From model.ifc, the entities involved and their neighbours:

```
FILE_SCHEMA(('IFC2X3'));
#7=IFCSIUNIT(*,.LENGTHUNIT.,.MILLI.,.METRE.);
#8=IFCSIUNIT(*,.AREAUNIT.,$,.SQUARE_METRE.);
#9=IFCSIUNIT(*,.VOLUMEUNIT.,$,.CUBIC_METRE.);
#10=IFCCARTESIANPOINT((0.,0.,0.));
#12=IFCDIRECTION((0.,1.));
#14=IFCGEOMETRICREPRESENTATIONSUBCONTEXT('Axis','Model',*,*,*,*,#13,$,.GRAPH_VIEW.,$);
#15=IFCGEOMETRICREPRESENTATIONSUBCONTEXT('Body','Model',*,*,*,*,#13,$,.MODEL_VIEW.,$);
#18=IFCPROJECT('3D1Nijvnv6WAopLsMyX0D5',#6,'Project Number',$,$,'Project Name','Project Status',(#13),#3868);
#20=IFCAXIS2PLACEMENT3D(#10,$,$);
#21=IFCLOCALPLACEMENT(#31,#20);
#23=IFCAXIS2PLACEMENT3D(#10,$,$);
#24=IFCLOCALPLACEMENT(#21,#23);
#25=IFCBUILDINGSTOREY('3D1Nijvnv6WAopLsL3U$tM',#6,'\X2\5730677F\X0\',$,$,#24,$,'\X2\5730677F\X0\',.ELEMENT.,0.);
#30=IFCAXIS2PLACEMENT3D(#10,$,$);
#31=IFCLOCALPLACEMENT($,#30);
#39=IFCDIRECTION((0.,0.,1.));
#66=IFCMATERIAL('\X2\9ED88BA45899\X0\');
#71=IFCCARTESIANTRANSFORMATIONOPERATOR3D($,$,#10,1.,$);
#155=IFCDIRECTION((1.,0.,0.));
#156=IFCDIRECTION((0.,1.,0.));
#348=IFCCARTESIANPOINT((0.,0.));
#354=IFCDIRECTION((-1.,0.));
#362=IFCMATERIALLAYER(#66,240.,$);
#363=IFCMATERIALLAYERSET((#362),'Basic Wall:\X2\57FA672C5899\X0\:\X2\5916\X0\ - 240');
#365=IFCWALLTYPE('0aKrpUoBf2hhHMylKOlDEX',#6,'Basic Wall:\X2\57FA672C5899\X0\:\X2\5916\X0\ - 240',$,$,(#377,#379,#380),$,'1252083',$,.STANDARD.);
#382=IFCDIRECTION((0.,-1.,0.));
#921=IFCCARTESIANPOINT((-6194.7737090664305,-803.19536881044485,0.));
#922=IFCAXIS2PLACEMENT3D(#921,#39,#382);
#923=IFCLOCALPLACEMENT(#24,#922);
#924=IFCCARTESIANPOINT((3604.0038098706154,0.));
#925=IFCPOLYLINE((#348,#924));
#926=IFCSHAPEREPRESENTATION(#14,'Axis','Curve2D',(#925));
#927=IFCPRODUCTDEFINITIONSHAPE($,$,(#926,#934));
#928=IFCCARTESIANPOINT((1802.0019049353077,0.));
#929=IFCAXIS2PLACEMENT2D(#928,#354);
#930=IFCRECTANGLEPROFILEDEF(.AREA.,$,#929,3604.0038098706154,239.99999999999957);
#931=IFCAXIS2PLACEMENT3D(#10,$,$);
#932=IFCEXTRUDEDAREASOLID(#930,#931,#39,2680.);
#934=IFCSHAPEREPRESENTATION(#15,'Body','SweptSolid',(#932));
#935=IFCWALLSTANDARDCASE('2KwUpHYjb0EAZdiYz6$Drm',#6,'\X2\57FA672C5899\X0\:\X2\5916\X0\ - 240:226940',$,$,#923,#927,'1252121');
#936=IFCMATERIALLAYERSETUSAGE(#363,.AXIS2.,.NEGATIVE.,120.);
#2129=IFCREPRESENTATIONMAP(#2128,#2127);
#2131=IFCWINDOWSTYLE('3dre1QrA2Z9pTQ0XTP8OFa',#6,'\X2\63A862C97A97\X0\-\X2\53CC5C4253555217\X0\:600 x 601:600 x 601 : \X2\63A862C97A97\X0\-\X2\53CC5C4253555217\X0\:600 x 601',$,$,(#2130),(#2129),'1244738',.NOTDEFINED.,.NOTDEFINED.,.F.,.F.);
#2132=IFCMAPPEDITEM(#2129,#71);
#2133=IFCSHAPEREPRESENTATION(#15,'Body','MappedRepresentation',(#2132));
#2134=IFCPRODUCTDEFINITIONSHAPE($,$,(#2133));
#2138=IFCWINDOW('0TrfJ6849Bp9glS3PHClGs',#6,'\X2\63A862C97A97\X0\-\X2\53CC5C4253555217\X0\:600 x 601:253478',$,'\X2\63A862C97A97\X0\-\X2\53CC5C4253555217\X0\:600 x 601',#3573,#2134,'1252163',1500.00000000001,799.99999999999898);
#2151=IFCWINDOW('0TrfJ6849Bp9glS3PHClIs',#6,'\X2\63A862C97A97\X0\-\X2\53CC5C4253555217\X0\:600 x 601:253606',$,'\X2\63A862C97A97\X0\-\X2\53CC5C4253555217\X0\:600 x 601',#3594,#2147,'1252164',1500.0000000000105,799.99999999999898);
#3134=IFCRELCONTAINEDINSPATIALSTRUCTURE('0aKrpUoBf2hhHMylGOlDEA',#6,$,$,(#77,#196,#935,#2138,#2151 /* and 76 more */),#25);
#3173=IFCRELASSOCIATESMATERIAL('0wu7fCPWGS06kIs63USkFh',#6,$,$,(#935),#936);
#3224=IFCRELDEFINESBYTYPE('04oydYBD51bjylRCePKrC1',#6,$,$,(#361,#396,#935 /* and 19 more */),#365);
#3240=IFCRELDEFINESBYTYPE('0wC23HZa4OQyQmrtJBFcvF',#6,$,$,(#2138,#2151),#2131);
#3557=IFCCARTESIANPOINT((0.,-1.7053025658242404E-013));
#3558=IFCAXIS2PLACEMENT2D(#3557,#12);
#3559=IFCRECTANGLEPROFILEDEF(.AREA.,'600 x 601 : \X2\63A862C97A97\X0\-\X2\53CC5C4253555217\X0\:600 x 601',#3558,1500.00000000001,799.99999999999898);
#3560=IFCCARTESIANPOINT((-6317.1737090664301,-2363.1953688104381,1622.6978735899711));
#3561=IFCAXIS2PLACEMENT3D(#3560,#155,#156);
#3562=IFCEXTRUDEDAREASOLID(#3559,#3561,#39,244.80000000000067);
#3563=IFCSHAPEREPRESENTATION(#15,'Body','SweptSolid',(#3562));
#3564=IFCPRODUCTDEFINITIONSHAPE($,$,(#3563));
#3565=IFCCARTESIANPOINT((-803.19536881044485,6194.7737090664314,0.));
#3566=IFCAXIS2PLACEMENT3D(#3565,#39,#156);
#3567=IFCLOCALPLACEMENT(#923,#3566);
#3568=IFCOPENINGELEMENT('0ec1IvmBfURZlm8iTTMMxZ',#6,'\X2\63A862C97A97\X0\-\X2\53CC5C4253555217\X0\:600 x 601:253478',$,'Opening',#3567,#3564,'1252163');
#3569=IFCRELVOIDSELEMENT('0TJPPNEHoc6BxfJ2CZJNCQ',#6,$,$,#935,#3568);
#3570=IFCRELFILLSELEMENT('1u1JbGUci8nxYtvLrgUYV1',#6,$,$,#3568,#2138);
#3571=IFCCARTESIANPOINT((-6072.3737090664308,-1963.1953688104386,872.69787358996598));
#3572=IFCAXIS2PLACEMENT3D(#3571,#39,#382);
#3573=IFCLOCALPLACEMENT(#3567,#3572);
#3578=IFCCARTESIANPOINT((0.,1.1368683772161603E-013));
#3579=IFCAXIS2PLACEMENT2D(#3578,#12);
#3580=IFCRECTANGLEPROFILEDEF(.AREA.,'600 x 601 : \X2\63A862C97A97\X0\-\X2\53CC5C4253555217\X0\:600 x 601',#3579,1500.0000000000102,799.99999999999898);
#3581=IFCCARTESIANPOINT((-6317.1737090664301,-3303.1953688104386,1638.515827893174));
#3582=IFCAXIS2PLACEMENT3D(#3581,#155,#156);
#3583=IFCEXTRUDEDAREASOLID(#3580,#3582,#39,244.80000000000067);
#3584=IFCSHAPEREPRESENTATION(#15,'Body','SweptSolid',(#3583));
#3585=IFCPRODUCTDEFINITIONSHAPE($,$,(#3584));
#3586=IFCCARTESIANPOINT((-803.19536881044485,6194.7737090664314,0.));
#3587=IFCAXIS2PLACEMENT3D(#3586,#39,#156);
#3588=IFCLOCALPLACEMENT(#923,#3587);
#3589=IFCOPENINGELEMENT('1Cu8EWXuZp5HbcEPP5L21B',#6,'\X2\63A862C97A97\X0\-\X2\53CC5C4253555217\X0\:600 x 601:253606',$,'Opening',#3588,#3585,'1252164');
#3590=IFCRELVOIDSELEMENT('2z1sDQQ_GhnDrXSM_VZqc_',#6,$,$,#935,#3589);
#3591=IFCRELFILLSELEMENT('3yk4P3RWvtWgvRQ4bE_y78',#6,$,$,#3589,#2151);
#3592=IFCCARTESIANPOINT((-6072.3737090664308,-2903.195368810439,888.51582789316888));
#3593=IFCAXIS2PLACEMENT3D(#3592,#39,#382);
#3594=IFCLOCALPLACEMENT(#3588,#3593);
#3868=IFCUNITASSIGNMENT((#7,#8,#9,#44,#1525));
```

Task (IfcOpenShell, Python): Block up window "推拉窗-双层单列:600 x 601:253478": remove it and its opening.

```python
import ifcopenshell
import ifcopenshell.api.feature
import ifcopenshell.api.root
import ifcopenshell.geom
import ifcopenshell.util.shape

model = ifcopenshell.open("model.ifc")
settings = ifcopenshell.geom.settings()


def volume(element):
    """Net volume in cubic metres, openings subtracted."""
    shape = ifcopenshell.geom.create_shape(settings, element)
    return ifcopenshell.util.shape.get_volume(shape.geometry)


window = model.by_guid("0TrfJ6849Bp9glS3PHClGs")
opening = window.FillsVoids[0].RelatingOpeningElement
wall = opening.VoidsElements[0].RelatingBuildingElement
before = volume(wall)

ifcopenshell.api.root.remove_product(model, product=window)
ifcopenshell.api.feature.remove_feature(model, feature=opening)

after = volume(wall)

print(f"wall volume {before:.3f} -> {after:.3f} m3")

model.write("model_edited.ifc")
```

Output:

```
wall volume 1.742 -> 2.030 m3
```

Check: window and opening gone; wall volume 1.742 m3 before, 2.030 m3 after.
